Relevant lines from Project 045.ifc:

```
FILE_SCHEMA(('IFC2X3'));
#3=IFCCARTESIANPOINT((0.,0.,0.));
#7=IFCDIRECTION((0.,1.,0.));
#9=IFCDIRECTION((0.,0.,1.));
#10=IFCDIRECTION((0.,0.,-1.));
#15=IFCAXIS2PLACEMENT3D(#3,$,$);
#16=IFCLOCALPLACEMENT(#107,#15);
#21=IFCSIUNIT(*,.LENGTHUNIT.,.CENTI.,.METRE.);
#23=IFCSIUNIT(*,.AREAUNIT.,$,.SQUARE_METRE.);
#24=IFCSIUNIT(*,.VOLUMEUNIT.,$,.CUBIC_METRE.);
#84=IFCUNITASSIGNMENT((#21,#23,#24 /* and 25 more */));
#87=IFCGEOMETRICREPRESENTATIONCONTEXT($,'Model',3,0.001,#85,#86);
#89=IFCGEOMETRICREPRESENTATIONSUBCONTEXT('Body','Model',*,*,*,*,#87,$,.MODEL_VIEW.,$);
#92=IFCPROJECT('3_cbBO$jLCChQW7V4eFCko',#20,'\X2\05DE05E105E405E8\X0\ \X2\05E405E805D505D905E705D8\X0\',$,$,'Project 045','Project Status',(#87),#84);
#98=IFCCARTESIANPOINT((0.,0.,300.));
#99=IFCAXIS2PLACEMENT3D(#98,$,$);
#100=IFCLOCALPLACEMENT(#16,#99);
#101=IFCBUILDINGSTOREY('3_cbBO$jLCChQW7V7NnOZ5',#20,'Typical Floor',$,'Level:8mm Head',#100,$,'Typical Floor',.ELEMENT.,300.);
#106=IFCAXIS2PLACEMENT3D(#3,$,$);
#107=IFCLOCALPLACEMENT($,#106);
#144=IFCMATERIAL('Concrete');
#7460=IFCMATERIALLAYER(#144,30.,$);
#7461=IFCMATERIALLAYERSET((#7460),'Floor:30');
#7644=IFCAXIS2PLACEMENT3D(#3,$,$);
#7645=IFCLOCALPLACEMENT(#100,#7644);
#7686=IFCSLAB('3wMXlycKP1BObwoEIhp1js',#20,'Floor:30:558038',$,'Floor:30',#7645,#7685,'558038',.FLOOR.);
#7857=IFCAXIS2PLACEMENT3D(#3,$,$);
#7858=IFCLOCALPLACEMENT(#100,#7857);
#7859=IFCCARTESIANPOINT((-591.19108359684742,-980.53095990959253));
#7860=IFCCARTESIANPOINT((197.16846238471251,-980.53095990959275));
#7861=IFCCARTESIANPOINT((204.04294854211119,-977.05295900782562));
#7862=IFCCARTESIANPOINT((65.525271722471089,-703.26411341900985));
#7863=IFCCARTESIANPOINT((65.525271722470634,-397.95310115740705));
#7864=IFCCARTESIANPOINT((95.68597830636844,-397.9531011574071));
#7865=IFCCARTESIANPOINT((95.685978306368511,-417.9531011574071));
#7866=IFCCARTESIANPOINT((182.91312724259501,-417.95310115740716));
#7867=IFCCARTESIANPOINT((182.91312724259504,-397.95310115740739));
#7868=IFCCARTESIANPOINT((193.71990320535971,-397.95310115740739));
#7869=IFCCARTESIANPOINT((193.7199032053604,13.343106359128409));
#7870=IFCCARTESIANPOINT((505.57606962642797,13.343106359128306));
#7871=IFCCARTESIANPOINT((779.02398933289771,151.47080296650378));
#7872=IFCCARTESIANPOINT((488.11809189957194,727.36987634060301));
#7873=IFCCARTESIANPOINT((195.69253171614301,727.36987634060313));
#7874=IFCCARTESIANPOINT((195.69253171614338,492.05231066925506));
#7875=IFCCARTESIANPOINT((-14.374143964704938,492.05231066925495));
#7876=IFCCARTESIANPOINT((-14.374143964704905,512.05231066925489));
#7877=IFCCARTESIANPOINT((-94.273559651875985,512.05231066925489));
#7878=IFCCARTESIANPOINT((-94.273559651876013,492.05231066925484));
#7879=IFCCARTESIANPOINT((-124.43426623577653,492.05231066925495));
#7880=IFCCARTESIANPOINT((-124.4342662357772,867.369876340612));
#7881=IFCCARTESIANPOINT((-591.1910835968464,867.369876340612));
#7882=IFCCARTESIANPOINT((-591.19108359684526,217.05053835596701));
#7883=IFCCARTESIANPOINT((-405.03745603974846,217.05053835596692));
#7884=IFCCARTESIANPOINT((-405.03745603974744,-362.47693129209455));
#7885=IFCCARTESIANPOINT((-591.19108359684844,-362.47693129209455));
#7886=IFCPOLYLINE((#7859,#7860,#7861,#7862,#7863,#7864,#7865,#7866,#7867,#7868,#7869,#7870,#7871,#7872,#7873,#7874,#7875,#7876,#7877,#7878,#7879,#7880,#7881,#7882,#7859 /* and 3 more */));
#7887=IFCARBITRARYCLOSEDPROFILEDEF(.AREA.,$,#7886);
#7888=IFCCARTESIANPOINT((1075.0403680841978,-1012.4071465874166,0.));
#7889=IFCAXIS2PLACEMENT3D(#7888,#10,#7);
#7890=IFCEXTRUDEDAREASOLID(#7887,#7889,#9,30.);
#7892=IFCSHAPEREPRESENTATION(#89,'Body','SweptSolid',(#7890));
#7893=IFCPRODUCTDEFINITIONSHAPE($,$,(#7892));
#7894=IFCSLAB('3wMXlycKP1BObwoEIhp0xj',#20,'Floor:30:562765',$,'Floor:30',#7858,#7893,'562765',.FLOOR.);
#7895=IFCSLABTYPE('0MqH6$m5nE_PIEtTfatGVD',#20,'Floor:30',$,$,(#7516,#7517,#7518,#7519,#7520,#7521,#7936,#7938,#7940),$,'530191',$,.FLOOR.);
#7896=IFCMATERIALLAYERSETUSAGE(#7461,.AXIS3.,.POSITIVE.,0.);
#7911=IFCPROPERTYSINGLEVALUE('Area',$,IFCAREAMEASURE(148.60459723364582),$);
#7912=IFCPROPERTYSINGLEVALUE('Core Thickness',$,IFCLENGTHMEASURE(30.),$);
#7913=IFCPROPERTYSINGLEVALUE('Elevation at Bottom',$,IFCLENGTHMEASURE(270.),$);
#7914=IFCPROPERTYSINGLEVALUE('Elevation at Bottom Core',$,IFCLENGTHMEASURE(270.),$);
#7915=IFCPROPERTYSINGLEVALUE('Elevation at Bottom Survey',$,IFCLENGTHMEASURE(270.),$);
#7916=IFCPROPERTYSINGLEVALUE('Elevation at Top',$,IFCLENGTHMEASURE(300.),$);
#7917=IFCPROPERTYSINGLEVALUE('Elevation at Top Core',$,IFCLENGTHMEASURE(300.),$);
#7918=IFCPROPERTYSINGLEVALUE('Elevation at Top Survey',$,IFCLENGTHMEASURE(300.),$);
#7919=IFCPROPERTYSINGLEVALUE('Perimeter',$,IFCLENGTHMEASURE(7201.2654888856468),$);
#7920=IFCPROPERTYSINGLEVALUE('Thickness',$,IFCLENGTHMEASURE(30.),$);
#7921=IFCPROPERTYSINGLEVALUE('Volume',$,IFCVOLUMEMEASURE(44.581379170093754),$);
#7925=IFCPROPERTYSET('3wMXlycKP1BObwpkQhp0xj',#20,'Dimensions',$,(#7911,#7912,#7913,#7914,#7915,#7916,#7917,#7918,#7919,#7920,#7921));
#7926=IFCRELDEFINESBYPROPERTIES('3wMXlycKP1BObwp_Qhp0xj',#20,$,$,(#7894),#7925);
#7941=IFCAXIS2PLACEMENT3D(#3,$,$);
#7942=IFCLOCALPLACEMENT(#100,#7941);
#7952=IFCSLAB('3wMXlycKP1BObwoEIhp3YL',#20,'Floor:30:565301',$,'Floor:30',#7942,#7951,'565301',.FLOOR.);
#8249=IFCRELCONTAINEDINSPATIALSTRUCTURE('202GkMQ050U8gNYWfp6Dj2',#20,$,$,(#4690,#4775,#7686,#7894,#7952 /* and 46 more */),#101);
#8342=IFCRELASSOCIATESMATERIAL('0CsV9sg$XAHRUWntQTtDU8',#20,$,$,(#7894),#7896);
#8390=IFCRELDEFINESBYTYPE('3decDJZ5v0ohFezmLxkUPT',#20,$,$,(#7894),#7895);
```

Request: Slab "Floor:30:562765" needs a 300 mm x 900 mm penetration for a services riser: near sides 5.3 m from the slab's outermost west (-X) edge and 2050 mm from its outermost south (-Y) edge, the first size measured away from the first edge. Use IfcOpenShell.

```python
import numpy as np
import ifcopenshell
import ifcopenshell.api.feature
import ifcopenshell.api.geometry
import ifcopenshell.api.pset
import ifcopenshell.api.root
import ifcopenshell.geom
import ifcopenshell.util.element
import ifcopenshell.util.placement
import ifcopenshell.util.representation
import ifcopenshell.util.shape
import ifcopenshell.util.unit

model = ifcopenshell.open("Project 045.ifc")
unit_scale = ifcopenshell.util.unit.calculate_unit_scale(model)
area_scale = ifcopenshell.util.unit.calculate_unit_scale(model, "AREAUNIT")
volume_scale = ifcopenshell.util.unit.calculate_unit_scale(model, "VOLUMEUNIT")
settings = ifcopenshell.geom.settings()


def volume(element):
    """Net volume in cubic metres, openings subtracted."""
    shape = ifcopenshell.geom.create_shape(settings, element)
    return ifcopenshell.util.shape.get_volume(shape.geometry)


slab = model.by_guid("3wMXlycKP1BObwoEIhp0xj")
before = volume(slab)

# Extent in the slab's own axes, in metres. The edges named are its -X and -Y sides.
slab_shape = ifcopenshell.geom.create_shape(settings, slab)
vertices = ifcopenshell.util.shape.get_vertices(slab_shape.geometry)
x_min, y_min, bottom = vertices.min(axis=0)
top = vertices[:, 2].max()

opening = ifcopenshell.api.root.create_entity(model, ifc_class="IfcOpeningElement", name="Services riser opening")
context = ifcopenshell.util.representation.get_context(model, "Model", "Body", "MODEL_VIEW")
width, depth = 0.3, 0.9
outline = [(0.0, 0.0), (width, 0.0), (width, depth), (0.0, depth), (0.0, 0.0)]
# Overshoot both faces by 50 mm so the cut is clean.
shape = ifcopenshell.api.geometry.add_slab_representation(
    model, context=context, depth=top - bottom + 0.1, polyline=outline
)
ifcopenshell.api.geometry.assign_representation(model, product=opening, representation=shape)

matrix = ifcopenshell.util.placement.get_local_placement(slab.ObjectPlacement)
matrix[:, 3] = matrix @ np.append(np.array([x_min + 5.3, y_min + 2.05, bottom - 0.05]) / unit_scale, 1.0)
ifcopenshell.api.geometry.edit_object_placement(model, product=opening, matrix=matrix, is_si=False)
ifcopenshell.api.feature.add_feature(model, feature=opening, element=slab)

after = volume(slab)

# Update the slab's stored quantities.
pset = model.by_id(ifcopenshell.util.element.get_pset(slab, "Dimensions", should_inherit=False)["id"])
ifcopenshell.api.pset.edit_pset(model, pset=pset, properties={
    "Area": model.create_entity("IfcAreaMeasure", after / (top - bottom) / area_scale),
    "Volume": model.create_entity("IfcVolumeMeasure", after / volume_scale),
})

print(f"slab volume {before:.3f} -> {after:.3f} m3")

model.write("Project 045_updated.ifc")
```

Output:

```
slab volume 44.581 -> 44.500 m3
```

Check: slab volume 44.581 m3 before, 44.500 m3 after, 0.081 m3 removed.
